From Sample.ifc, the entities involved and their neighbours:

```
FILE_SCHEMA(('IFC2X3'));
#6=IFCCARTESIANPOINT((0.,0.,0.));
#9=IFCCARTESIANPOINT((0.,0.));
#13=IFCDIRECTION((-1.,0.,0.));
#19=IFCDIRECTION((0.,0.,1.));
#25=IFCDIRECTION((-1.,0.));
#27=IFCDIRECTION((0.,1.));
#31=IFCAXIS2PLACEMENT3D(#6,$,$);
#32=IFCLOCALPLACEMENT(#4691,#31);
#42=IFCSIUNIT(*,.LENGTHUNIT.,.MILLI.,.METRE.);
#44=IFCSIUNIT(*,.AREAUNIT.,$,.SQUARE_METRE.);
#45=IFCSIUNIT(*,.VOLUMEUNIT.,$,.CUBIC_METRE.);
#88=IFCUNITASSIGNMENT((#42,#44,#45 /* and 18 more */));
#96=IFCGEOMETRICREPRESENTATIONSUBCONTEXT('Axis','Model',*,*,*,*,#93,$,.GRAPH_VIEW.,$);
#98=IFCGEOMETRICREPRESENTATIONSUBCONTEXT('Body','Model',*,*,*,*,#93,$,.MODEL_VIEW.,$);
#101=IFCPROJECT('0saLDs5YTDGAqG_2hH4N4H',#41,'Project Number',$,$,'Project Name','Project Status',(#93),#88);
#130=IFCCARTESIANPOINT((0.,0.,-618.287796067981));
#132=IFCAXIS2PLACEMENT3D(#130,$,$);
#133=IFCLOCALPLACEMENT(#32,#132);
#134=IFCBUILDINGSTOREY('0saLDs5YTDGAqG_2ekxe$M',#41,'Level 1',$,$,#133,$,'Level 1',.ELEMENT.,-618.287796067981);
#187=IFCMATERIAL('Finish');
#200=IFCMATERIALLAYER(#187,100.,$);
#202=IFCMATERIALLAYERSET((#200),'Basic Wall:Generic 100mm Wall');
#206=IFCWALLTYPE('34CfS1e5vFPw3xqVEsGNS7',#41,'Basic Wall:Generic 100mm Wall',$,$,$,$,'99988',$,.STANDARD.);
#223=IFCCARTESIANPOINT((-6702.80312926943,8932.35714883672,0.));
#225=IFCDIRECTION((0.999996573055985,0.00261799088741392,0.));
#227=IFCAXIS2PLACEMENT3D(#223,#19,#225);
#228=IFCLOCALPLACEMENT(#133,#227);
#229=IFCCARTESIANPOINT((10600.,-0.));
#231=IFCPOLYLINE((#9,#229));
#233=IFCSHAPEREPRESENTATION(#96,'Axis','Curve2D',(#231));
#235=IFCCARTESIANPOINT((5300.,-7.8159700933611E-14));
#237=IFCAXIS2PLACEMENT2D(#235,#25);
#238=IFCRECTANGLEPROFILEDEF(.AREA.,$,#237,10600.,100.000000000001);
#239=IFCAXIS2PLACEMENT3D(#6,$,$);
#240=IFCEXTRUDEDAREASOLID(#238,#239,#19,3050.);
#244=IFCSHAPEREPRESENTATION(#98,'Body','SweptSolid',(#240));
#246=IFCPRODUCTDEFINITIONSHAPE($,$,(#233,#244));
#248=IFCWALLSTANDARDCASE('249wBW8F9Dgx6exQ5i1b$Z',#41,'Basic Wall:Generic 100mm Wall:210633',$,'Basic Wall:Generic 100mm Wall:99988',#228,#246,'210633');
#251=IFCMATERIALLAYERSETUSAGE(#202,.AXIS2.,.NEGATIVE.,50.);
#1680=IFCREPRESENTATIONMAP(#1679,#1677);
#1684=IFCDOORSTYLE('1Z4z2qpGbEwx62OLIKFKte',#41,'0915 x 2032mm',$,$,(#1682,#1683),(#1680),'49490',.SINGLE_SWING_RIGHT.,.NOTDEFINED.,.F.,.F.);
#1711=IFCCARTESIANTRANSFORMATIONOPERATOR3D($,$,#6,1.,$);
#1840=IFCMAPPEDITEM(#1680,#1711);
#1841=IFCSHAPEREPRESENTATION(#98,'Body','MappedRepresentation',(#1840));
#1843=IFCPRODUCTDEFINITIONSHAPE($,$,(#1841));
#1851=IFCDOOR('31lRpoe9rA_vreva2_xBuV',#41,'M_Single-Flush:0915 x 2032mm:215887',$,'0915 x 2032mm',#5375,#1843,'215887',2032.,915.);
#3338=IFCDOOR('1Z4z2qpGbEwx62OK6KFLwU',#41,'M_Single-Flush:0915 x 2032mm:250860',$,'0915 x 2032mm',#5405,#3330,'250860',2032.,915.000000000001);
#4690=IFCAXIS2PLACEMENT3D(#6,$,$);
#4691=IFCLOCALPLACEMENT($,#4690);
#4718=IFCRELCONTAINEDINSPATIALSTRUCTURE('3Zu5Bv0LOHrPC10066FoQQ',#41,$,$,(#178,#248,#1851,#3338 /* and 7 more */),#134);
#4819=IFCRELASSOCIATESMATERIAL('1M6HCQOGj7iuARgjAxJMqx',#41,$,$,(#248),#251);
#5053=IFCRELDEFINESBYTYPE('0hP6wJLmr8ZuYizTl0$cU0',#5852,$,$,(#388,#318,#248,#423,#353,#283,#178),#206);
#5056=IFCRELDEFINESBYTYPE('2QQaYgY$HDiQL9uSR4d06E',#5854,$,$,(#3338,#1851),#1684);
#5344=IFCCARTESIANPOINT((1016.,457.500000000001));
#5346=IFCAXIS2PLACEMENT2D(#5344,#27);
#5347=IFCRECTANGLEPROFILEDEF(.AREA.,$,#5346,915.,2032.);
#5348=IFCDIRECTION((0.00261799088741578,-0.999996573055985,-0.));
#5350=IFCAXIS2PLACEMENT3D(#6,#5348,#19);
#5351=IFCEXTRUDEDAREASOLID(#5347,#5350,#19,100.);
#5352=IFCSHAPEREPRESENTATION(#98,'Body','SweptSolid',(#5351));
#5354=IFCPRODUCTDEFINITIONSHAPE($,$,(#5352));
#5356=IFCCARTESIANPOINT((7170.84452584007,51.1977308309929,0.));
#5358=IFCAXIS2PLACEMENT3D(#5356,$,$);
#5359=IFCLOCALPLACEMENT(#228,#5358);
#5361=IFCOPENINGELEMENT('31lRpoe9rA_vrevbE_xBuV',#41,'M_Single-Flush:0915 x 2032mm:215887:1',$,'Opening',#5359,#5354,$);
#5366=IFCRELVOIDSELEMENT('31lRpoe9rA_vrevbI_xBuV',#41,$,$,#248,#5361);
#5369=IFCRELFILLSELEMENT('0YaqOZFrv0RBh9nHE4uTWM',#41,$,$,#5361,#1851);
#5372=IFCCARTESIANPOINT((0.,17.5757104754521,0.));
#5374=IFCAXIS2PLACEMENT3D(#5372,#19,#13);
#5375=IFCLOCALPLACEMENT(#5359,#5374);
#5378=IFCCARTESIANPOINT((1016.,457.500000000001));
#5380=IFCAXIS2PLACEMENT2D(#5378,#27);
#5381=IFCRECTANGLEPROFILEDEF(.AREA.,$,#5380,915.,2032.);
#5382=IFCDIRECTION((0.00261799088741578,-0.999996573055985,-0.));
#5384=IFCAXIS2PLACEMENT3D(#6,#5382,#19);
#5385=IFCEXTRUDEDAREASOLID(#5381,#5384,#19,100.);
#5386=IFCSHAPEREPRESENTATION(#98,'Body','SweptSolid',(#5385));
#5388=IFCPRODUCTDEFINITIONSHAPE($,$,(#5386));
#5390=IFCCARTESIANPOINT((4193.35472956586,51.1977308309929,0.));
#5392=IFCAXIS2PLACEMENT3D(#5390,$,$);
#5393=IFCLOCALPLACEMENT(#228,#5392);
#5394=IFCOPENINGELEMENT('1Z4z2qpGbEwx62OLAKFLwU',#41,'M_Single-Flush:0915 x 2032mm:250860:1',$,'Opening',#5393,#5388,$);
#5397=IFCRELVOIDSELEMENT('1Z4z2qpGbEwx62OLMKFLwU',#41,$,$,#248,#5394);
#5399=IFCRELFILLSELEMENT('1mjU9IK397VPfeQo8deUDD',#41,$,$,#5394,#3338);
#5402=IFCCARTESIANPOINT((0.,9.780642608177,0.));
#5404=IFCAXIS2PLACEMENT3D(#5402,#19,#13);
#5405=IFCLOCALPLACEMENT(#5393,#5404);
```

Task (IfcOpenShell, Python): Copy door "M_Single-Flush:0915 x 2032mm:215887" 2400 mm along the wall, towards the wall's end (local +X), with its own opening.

```python
import ifcopenshell
import ifcopenshell.api.feature
import ifcopenshell.api.geometry
import ifcopenshell.api.root
import ifcopenshell.geom
import ifcopenshell.util.element
import ifcopenshell.util.placement
import ifcopenshell.util.shape

model = ifcopenshell.open("Sample.ifc")
settings = ifcopenshell.geom.settings()


def volume(element):
    """Net volume in cubic metres, openings subtracted."""
    shape = ifcopenshell.geom.create_shape(settings, element)
    return ifcopenshell.util.shape.get_volume(shape.geometry)


def reuse_history(source, copy):
    """copy_class also copies each property set's owner history, people and application; keep the originals."""
    for rel in copy.IsDefinedBy:
        if rel.is_a("IfcRelDefinesByProperties") and (history := rel.RelatingPropertyDefinition.OwnerHistory):
            rel.RelatingPropertyDefinition.OwnerHistory = source.OwnerHistory
            ifcopenshell.util.element.remove_deep2(model, history)


door = model.by_guid("31lRpoe9rA_vreva2_xBuV")
opening = door.FillsVoids[0].RelatingOpeningElement
wall = opening.VoidsElements[0].RelatingBuildingElement
before = volume(wall)
shift = ifcopenshell.util.placement.get_local_placement(wall.ObjectPlacement)[:3, 0] * 2400.0

# copy_class copies the void relationship, type, container and properties, but no geometry.
new_opening = ifcopenshell.api.root.copy_class(model, product=opening)
new_opening.Representation = ifcopenshell.util.element.copy_deep(
    model, opening.Representation, exclude=["IfcGeometricRepresentationContext", "IfcRepresentationMap"]
)
new_opening.Name = "M_Single-Flush:0915 x 2032mm"
new_door = ifcopenshell.api.root.copy_class(model, product=door)
new_door.Representation = ifcopenshell.util.element.copy_deep(
    model, door.Representation, exclude=["IfcGeometricRepresentationContext", "IfcRepresentationMap"]
)
new_door.Name = "M_Single-Flush:0915 x 2032mm"
new_door.Tag = None
reuse_history(door, new_door)
fills = ifcopenshell.api.feature.add_filling(model, opening=new_opening, element=new_door)
fills.OwnerHistory = new_door.OwnerHistory  # required in IFC2X3

for old, new in ((opening, new_opening), (door, new_door)):
    matrix = ifcopenshell.util.placement.get_local_placement(old.ObjectPlacement)
    matrix[:3, 3] += shift
    ifcopenshell.api.geometry.edit_object_placement(model, product=new, matrix=matrix, is_si=False)

after = volume(wall)

print(f"wall volume {before:.3f} -> {after:.3f} m3")

model.write("Sample-out.ifc")
```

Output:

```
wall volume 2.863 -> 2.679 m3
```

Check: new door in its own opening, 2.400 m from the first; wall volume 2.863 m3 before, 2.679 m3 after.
